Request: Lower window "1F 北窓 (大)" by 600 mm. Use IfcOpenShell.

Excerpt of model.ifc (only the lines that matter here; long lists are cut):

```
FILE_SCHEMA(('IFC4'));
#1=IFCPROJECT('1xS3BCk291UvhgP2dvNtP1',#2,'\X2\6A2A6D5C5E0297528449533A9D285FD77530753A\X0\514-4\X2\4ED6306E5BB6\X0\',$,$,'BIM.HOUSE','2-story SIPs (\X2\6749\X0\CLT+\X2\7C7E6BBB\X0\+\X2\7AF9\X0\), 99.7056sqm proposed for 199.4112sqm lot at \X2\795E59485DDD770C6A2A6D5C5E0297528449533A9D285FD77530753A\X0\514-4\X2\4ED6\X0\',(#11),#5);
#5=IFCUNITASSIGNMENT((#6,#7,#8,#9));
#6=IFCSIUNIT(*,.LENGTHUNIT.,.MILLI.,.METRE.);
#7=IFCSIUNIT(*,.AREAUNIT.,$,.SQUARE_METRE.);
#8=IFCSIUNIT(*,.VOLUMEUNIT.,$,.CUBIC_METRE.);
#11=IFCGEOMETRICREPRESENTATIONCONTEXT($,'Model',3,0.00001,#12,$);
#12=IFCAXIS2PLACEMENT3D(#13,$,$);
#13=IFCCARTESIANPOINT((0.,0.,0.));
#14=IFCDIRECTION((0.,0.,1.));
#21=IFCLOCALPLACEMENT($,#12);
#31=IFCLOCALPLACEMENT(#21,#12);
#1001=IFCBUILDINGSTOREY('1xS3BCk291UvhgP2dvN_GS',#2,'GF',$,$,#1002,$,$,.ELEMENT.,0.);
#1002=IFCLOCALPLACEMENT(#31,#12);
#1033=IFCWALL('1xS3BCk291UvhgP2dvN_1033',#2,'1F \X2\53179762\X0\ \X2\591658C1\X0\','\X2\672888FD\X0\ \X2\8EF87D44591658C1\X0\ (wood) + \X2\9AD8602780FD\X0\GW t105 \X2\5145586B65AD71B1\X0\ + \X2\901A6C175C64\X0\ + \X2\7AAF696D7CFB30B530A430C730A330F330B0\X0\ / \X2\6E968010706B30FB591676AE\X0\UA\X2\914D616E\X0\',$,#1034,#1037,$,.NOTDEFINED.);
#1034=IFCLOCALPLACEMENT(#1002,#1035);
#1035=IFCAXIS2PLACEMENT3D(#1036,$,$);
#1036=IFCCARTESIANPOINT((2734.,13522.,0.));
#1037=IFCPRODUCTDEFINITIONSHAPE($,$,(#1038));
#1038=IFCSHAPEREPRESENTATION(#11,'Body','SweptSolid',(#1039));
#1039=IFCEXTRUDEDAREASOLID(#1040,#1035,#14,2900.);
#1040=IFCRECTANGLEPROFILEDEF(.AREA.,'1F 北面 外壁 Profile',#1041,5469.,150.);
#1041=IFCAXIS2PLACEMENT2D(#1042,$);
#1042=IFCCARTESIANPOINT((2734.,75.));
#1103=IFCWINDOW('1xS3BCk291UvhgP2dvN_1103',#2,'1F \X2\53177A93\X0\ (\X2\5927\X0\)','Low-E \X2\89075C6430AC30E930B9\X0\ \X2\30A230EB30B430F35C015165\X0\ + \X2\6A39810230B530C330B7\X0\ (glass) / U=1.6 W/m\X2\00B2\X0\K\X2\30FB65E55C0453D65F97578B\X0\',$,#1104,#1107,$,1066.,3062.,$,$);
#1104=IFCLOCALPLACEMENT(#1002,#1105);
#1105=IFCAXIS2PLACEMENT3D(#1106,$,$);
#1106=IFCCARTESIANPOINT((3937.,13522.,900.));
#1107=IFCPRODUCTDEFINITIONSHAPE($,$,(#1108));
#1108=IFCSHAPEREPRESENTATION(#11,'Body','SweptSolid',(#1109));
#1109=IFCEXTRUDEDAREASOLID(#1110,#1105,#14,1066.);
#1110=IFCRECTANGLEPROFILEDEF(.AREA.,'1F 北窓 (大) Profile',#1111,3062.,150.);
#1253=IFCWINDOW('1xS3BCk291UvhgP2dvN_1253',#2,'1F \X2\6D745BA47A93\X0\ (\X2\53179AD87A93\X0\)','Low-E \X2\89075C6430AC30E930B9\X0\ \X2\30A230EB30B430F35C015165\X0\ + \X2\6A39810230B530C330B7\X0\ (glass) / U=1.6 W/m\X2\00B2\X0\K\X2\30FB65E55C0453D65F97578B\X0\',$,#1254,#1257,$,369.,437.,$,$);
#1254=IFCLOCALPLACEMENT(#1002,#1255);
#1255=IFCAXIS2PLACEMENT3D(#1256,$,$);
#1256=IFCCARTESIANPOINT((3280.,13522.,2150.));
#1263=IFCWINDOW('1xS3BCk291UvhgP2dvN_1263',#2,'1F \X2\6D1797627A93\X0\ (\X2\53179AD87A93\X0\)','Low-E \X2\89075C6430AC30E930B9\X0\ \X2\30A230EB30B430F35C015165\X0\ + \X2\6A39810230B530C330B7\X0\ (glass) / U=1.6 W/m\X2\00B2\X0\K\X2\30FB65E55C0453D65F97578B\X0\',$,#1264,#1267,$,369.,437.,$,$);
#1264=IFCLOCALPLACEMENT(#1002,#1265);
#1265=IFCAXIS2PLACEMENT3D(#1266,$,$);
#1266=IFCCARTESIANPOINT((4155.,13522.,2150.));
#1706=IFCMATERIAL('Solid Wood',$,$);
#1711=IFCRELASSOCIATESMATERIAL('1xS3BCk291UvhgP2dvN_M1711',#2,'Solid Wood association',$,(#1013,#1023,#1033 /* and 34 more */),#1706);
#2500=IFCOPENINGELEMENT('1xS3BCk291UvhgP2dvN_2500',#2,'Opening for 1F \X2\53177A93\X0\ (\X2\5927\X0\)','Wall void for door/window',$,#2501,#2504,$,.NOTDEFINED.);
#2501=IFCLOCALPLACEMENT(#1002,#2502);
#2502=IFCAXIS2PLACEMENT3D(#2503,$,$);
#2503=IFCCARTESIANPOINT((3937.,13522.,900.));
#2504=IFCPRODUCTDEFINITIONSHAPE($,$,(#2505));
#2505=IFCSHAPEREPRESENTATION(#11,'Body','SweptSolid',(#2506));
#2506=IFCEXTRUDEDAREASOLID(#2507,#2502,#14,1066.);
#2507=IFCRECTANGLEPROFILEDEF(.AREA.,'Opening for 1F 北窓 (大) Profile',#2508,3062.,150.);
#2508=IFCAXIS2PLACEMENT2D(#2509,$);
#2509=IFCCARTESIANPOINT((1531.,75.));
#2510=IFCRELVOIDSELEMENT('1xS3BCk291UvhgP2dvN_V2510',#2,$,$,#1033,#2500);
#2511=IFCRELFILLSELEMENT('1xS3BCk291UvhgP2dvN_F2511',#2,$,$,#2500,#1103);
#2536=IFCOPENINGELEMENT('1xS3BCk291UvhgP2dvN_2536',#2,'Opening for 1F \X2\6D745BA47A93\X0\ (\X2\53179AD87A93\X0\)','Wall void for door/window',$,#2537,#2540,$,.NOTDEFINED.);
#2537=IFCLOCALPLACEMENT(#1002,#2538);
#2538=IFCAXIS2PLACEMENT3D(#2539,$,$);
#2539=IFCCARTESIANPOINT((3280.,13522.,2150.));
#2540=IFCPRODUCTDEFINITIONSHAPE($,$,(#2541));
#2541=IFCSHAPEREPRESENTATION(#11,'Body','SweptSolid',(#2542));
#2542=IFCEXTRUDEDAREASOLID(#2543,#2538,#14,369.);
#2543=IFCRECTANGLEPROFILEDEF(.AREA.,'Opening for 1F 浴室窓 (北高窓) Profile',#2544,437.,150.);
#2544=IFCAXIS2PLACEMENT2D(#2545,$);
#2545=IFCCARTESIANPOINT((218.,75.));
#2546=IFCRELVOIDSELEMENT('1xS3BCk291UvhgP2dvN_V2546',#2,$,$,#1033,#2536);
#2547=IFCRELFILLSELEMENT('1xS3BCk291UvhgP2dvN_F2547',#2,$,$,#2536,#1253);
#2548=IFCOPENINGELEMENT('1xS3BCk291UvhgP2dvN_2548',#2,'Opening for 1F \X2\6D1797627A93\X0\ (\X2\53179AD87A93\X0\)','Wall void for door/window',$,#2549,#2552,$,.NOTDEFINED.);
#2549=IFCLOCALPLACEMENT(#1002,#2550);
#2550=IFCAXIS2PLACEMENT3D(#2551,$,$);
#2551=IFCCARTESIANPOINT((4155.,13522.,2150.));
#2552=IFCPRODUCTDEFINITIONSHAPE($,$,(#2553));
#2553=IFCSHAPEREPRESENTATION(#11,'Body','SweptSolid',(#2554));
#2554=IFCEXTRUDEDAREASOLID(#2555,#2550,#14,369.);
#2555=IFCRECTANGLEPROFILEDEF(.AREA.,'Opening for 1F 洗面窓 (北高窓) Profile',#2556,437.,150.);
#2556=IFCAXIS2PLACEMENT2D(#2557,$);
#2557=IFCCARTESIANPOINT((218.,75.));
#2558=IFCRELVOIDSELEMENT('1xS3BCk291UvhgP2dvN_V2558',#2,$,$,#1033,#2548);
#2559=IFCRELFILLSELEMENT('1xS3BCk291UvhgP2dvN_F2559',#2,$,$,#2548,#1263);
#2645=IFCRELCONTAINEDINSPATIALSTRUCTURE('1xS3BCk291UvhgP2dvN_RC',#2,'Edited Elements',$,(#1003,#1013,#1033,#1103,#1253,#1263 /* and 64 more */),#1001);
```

```python
import numpy as np
import ifcopenshell
import ifcopenshell.api.geometry
import ifcopenshell.util.placement
import ifcopenshell.util.unit

model = ifcopenshell.open("model.ifc")
unit_scale = ifcopenshell.util.unit.calculate_unit_scale(model)

window = model.by_guid("1xS3BCk291UvhgP2dvN_1103")
opening = window.FillsVoids[0].RelatingOpeningElement
dz = -600.0

shift = np.array([0.0, 0.0, dz])
# The window is not placed relative to its opening, so move both.
for product in (opening, window):
    matrix = ifcopenshell.util.placement.get_local_placement(product.ObjectPlacement)
    matrix[:3, 3] += shift
    ifcopenshell.api.geometry.edit_object_placement(model, product=product, matrix=matrix, is_si=False)

print(f"moved by {dz * unit_scale:+.3f} m")

model.write("model_v2.ifc")
```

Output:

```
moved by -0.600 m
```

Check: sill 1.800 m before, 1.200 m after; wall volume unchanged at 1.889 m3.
